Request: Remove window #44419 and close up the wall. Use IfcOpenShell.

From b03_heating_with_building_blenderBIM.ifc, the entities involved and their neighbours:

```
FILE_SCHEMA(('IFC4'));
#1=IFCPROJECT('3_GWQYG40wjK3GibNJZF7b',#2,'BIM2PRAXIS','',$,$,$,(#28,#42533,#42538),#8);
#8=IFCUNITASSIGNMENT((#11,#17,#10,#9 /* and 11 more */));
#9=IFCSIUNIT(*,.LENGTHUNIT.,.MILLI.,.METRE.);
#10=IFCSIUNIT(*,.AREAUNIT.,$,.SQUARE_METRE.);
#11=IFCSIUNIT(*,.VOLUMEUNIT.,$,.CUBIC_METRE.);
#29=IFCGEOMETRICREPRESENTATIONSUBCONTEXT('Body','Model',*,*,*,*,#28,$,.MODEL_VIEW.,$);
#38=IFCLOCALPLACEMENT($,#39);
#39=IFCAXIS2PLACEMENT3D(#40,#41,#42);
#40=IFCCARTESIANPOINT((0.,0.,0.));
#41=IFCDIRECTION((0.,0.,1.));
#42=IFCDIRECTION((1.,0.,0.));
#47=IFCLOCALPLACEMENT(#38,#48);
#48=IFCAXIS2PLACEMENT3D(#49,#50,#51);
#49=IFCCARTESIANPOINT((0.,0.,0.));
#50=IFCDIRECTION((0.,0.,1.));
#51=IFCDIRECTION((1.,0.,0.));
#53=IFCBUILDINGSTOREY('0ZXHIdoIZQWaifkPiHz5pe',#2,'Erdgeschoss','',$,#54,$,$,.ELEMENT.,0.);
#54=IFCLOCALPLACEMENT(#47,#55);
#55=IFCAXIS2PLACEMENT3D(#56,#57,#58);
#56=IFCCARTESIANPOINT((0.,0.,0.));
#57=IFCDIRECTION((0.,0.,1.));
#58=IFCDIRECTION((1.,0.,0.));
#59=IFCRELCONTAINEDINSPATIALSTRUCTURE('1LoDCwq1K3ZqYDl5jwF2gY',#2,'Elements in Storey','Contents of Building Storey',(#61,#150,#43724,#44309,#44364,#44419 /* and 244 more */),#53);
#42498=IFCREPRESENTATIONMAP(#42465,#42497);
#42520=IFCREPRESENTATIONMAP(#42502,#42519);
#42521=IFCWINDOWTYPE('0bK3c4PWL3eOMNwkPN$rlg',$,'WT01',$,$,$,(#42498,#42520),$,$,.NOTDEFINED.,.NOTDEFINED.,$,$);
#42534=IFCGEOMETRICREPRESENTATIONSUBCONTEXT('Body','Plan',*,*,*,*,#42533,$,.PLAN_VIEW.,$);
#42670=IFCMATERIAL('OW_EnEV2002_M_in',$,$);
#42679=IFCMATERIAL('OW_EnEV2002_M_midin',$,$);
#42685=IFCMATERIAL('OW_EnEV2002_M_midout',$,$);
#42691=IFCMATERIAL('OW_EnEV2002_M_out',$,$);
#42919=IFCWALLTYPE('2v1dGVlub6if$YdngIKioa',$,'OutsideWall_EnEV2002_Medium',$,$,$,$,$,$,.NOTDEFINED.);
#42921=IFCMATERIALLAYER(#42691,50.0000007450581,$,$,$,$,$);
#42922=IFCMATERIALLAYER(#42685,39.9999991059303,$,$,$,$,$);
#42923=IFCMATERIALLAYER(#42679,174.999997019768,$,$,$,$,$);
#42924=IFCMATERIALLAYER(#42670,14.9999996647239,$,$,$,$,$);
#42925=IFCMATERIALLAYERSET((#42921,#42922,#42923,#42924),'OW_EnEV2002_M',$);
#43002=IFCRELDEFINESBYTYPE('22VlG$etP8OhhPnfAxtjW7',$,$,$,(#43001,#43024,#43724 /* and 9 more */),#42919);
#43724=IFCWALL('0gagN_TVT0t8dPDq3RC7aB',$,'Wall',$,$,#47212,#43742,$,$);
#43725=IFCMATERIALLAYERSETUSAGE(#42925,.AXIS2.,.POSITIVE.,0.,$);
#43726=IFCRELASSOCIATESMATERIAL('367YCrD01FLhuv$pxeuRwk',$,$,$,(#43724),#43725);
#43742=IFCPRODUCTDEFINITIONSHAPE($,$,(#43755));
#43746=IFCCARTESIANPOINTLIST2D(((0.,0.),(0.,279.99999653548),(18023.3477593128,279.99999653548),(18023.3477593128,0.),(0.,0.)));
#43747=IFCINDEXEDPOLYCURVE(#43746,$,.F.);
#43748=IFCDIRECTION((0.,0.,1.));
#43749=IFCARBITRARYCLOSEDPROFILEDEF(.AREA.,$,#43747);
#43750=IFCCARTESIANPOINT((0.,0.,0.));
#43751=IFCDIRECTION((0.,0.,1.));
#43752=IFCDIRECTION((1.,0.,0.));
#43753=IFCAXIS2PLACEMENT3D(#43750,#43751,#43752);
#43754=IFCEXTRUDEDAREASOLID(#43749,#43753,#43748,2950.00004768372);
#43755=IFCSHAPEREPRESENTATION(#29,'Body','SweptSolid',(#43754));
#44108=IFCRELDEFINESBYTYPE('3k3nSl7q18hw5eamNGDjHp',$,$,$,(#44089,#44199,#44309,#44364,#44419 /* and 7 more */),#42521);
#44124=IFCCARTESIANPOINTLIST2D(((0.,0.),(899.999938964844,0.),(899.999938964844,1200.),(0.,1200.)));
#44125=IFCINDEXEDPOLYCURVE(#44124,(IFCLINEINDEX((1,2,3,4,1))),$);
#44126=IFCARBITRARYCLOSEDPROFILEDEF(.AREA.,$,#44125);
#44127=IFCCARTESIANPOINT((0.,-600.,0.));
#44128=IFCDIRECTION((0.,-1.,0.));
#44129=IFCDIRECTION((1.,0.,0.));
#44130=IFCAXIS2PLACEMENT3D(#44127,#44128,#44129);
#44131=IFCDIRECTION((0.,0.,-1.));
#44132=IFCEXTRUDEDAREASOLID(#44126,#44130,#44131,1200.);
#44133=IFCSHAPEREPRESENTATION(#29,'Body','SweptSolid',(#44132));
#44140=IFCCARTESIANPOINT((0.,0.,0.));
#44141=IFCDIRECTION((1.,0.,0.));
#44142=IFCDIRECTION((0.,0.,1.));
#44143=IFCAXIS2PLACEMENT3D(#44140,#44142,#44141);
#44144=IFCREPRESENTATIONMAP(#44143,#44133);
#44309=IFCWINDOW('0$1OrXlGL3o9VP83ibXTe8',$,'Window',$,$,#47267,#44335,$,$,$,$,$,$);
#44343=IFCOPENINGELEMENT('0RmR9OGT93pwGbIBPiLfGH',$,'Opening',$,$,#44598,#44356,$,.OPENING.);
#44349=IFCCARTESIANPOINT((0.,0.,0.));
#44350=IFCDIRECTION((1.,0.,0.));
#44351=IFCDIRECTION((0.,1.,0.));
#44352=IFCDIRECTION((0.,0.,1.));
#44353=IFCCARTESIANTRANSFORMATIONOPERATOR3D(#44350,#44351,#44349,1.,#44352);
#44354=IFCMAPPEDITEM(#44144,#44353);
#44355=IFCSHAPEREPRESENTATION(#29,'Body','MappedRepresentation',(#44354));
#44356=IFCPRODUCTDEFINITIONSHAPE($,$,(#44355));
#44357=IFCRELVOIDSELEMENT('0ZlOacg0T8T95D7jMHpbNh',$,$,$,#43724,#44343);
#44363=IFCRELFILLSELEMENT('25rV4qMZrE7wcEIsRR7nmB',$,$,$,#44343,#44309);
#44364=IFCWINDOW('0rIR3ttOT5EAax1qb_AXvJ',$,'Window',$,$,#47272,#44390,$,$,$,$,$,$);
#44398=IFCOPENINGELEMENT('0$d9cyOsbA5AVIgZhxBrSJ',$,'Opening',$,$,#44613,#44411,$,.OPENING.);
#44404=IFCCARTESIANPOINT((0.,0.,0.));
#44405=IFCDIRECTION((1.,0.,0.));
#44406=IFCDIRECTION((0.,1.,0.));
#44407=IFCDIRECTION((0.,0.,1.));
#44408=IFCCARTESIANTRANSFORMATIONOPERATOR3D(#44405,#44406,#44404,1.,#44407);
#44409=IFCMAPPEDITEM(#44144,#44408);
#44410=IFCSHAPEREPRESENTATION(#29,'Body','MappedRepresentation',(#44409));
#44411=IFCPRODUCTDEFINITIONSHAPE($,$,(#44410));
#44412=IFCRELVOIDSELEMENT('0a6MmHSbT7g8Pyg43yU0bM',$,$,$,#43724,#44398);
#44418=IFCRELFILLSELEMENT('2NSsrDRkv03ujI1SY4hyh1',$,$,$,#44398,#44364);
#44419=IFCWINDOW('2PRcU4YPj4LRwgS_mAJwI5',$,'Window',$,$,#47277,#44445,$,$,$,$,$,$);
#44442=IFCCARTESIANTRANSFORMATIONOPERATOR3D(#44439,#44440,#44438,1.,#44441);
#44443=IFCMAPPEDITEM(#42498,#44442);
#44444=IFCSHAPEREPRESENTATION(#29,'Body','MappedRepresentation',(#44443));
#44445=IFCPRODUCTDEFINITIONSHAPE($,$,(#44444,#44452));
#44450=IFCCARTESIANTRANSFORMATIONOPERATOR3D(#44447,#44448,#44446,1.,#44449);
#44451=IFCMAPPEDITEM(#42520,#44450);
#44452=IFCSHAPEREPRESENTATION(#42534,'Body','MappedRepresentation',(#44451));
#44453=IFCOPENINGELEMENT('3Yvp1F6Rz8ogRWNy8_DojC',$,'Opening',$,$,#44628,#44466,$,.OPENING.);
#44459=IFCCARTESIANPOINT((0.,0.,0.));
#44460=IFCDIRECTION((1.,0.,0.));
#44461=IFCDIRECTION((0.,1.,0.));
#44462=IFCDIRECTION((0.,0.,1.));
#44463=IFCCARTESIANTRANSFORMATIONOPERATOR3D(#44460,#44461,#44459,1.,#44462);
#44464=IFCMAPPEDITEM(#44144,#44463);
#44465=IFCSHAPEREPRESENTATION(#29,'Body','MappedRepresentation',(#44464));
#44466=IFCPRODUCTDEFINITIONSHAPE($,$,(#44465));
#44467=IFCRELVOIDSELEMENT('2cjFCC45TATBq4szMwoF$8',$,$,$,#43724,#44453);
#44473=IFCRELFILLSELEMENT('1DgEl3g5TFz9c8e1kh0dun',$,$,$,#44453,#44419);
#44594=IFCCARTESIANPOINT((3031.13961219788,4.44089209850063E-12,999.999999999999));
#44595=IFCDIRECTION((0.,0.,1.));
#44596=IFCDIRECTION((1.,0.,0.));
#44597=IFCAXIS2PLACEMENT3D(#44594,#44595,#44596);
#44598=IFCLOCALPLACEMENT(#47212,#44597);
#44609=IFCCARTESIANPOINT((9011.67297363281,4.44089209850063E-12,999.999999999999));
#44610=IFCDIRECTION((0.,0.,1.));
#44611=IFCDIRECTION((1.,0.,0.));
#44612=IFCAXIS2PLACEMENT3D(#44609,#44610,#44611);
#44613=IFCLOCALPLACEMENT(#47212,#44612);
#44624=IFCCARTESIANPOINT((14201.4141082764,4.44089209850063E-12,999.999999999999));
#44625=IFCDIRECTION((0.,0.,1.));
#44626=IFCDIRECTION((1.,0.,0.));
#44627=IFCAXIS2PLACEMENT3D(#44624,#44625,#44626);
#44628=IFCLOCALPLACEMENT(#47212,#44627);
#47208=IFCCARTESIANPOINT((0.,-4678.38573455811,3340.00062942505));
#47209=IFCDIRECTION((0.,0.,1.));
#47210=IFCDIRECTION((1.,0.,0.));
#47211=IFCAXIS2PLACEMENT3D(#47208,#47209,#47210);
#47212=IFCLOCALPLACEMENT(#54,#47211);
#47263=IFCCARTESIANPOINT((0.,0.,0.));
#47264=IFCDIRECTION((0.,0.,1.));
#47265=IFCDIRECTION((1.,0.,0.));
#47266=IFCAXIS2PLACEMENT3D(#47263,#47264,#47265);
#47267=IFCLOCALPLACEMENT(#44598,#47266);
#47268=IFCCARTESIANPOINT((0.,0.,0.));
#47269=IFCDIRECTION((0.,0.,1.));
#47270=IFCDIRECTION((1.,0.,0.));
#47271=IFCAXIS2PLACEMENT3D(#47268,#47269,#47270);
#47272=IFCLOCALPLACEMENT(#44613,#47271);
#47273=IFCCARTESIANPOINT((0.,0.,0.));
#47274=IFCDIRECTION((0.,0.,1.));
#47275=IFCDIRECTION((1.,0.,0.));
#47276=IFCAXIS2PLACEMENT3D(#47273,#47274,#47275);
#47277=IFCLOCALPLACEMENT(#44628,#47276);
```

```python
import ifcopenshell
import ifcopenshell.api.feature
import ifcopenshell.api.root
import ifcopenshell.geom
import ifcopenshell.util.shape

model = ifcopenshell.open("b03_heating_with_building_blenderBIM.ifc")
settings = ifcopenshell.geom.settings()


def volume(element):
    """Net volume in cubic metres, openings subtracted."""
    shape = ifcopenshell.geom.create_shape(settings, element)
    return ifcopenshell.util.shape.get_volume(shape.geometry)


window = model.by_guid("2PRcU4YPj4LRwgS_mAJwI5")
opening = window.FillsVoids[0].RelatingOpeningElement
wall = opening.VoidsElements[0].RelatingBuildingElement
before = volume(wall)

ifcopenshell.api.root.remove_product(model, product=window)
ifcopenshell.api.feature.remove_feature(model, feature=opening)

after = volume(wall)

print(f"wall volume {before:.3f} -> {after:.3f} m3")

model.write("b03_heating_with_building_blenderBIM-out.ifc")
```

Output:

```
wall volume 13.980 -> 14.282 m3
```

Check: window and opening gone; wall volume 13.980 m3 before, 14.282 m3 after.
